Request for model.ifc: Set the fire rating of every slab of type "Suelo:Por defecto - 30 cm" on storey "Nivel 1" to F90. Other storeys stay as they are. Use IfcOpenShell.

First a look at what the model holds.

```python
import ifcopenshell
import ifcopenshell.util.element

model = ifcopenshell.open("model.ifc")
print(model.schema)
storey = next(s for s in model.by_type("IfcBuildingStorey") if s.Name == "Nivel 1")
slabs = [e for e in ifcopenshell.util.element.get_decomposition(storey) if e.is_a("IfcSlab")]
seen = {}
for e in slabs:
    element_type = ifcopenshell.util.element.get_type(e)
    key = (element_type.Name if element_type != e and element_type else None, ifcopenshell.util.element.get_pset(e, "Pset_SlabCommon", "FireRating"))
    seen[key] = seen.get(key, 0) + 1
for (name, value), count in sorted(seen.items(), key=str):
    print(count, "x", name, "|", value)
```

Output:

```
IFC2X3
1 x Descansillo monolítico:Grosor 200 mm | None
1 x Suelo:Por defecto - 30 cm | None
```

```python
import ifcopenshell
import ifcopenshell.api.pset
import ifcopenshell.util.element

model = ifcopenshell.open("model.ifc")

storey = next(s for s in model.by_type("IfcBuildingStorey") if s.Name == "Nivel 1")
slabs = [e for e in ifcopenshell.util.element.get_decomposition(storey) if e.is_a("IfcSlab")]

count = 0
for e in slabs:
    element_type = ifcopenshell.util.element.get_type(e)
    if element_type in (None, e) or element_type.Name != "Suelo:Por defecto - 30 cm":
        continue
    # add_pset returns the element's existing set when there is one.
    pset = ifcopenshell.api.pset.add_pset(model, product=e, name="Pset_SlabCommon")
    ifcopenshell.api.pset.edit_pset(model, pset=pset, properties={"FireRating": "F90"})
    count += 1

print(count, "slabs updated")

model.write("model_v2.ifc")
```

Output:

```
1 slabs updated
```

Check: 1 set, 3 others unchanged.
